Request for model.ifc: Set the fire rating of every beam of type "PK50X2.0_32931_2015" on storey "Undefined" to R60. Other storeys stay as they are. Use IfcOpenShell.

First a look at what the model holds.

```python
import ifcopenshell
import ifcopenshell.util.element

model = ifcopenshell.open("model.ifc")
print(model.schema)
storey = next(s for s in model.by_type("IfcBuildingStorey") if s.Name == "Undefined")
beams = [e for e in ifcopenshell.util.element.get_decomposition(storey) if e.is_a("IfcBeam")]
seen = {}
for e in beams:
    element_type = ifcopenshell.util.element.get_type(e)
    key = (element_type.Name if element_type != e and element_type else None, ifcopenshell.util.element.get_pset(e, "Pset_BeamCommon", "FireRating"))
    seen[key] = seen.get(key, 0) + 1
for (name, value), count in sorted(seen.items(), key=str):
    print(count, "x", name, "|", value)
```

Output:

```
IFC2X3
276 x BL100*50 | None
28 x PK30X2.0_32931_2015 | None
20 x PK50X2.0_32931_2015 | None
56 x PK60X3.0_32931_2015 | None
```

```python
import ifcopenshell
import ifcopenshell.api.pset
import ifcopenshell.util.element

model = ifcopenshell.open("model.ifc")

storey = next(s for s in model.by_type("IfcBuildingStorey") if s.Name == "Undefined")
beams = [e for e in ifcopenshell.util.element.get_decomposition(storey) if e.is_a("IfcBeam")]

count = 0
for e in beams:
    element_type = ifcopenshell.util.element.get_type(e)
    if element_type in (None, e) or element_type.Name != "PK50X2.0_32931_2015":
        continue
    found = ifcopenshell.util.element.get_pset(e, "Pset_BeamCommon", should_inherit=False)
    if found:
        pset = model.by_id(found["id"])
        if len(ifcopenshell.util.element.get_elements_by_pset(pset)) > 1:
            pset = ifcopenshell.api.pset.unshare_pset(model, products=[e], pset=pset)[0]
    else:
        pset = ifcopenshell.api.pset.add_pset(model, product=e, name="Pset_BeamCommon")
    ifcopenshell.api.pset.edit_pset(model, pset=pset, properties={"FireRating": "R60"})
    count += 1

print(count, "beams updated")

model.write("model_edited.ifc")
```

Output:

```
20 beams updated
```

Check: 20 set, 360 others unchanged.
